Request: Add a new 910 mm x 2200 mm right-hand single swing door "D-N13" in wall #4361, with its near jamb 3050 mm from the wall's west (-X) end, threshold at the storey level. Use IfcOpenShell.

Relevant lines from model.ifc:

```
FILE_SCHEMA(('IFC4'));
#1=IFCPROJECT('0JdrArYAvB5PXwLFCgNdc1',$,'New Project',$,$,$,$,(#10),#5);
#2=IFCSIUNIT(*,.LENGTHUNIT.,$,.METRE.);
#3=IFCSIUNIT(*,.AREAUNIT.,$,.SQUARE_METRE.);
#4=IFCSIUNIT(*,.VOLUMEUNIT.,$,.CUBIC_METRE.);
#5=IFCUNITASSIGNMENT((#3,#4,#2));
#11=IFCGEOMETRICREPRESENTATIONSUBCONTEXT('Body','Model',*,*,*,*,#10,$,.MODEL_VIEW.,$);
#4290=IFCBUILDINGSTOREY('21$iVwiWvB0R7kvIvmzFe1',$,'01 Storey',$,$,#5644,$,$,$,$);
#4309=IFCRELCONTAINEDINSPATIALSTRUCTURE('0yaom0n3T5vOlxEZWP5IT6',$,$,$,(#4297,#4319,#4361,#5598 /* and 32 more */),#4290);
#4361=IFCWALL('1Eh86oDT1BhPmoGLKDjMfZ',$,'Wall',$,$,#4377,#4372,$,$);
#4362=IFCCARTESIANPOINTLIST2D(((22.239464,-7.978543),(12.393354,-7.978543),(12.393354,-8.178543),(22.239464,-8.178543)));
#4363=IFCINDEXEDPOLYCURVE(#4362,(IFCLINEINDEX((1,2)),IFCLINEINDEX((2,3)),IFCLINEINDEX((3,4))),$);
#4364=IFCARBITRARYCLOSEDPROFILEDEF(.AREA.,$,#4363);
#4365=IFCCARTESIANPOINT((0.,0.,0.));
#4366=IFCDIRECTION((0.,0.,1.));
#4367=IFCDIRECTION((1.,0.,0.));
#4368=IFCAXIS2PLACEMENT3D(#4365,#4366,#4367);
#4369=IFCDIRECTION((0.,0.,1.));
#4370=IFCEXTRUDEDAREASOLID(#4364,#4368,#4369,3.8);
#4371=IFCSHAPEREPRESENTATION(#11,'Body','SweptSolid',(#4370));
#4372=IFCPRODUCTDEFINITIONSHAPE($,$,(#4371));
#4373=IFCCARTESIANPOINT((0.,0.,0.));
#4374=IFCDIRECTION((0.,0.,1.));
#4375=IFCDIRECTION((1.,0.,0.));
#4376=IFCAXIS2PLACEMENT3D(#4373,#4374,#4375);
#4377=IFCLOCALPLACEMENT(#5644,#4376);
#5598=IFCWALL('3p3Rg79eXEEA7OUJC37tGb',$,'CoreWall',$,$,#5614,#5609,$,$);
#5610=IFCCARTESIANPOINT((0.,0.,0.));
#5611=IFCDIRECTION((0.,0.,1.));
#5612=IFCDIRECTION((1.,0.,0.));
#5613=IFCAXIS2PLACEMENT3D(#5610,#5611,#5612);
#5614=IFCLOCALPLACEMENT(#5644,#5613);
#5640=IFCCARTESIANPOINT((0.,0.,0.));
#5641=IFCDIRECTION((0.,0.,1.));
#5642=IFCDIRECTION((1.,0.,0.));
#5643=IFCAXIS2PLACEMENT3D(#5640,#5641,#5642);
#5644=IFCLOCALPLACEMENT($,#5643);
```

```python
import numpy as np
import ifcopenshell
import ifcopenshell.api.feature
import ifcopenshell.api.geometry
import ifcopenshell.api.root
import ifcopenshell.api.spatial
import ifcopenshell.geom
import ifcopenshell.util.element
import ifcopenshell.util.placement
import ifcopenshell.util.representation
import ifcopenshell.util.shape
import ifcopenshell.util.unit

model = ifcopenshell.open("model.ifc")
unit_scale = ifcopenshell.util.unit.calculate_unit_scale(model)
settings = ifcopenshell.geom.settings()


def volume(element):
    """Net volume in cubic metres, openings subtracted."""
    shape = ifcopenshell.geom.create_shape(settings, element)
    return ifcopenshell.util.shape.get_volume(shape.geometry)


wall = model.by_guid("1Eh86oDT1BhPmoGLKDjMfZ")
storey = ifcopenshell.util.element.get_container(wall, ifc_class="IfcBuildingStorey")
context = ifcopenshell.util.representation.get_context(model, "Model", "Body", "MODEL_VIEW")
before = volume(wall)

width, height, from_end, sill = 0.91, 2.2, 3.05, 0.0  # metres

# The wall runs along its own X axis, and the end named is its -X end.
wall_shape = ifcopenshell.geom.create_shape(settings, wall)
x, y, z = ifcopenshell.util.shape.get_vertices(wall_shape.geometry).T
start = x.min() + from_end
face, thickness = float(y.min()), float(y.max() - y.min())
wall_matrix = ifcopenshell.util.placement.get_local_placement(wall.ObjectPlacement)
level = ifcopenshell.util.placement.get_local_placement(storey.ObjectPlacement)[2, 3]


def in_wall(x, y):
    """Placement at x, y metres in the wall's axes, at sill height."""
    matrix = wall_matrix.copy()
    matrix[:, 3] = wall_matrix @ np.array([x / unit_scale, y / unit_scale, 0.0, 1.0])
    matrix[2, 3] = level + sill / unit_scale
    return matrix


# Opening: a box that overshoots both wall faces by 50 mm.
opening = ifcopenshell.api.root.create_entity(model, ifc_class="IfcOpeningElement", predefined_type="OPENING")
box = ifcopenshell.api.geometry.add_wall_representation(
    model, context=context, length=width, height=height, thickness=thickness + 0.1
)
ifcopenshell.api.geometry.assign_representation(model, product=opening, representation=box)
ifcopenshell.api.geometry.edit_object_placement(model, product=opening, matrix=in_wall(start, face - 0.05), is_si=False)
ifcopenshell.api.feature.add_feature(model, feature=opening, element=wall)

door = ifcopenshell.api.root.create_entity(model, ifc_class="IfcDoor", name="D-N13", predefined_type="DOOR")
door.OverallWidth, door.OverallHeight = width / unit_scale, height / unit_scale
door.OperationType = "SINGLE_SWING_RIGHT"
body = ifcopenshell.api.geometry.add_door_representation(
    model,
    context=context,
    overall_width=door.OverallWidth,
    overall_height=door.OverallHeight,
    operation_type="SINGLE_SWING_RIGHT",
    lining_properties={"LiningDepth": thickness / unit_scale, "ThresholdDepth": thickness / unit_scale},
)
ifcopenshell.api.geometry.assign_representation(model, product=door, representation=body)
ifcopenshell.api.spatial.assign_container(model, products=[door], relating_structure=storey)
ifcopenshell.api.feature.add_filling(model, opening=opening, element=door)

# The lining spans the wall, so the door starts at the wall face.
ifcopenshell.api.geometry.edit_object_placement(model, product=door, matrix=in_wall(start, face), is_si=False)

after = volume(wall)

print(f"wall volume {before:.3f} -> {after:.3f} m3")

model.write("model_v2.ifc")
```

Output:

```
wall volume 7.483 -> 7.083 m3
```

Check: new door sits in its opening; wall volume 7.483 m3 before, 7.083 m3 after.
